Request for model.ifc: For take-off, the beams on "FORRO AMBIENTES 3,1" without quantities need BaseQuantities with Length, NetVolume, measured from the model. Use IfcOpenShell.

First a look at what the model holds.

```python
import ifcopenshell
import ifcopenshell.util.element
import ifcopenshell.util.unit

model = ifcopenshell.open("model.ifc")
print(model.schema)
for unit_type in ("LENGTHUNIT", "AREAUNIT", "VOLUMEUNIT"):
    print(unit_type, ifcopenshell.util.unit.calculate_unit_scale(model, unit_type))
storey = next(s for s in model.by_type("IfcBuildingStorey") if s.Name == "FORRO AMBIENTES 3,1")
beams = [e for e in ifcopenshell.util.element.get_decomposition(storey) if e.is_a("IfcBeam")]
for e in sorted(beams, key=lambda e: e.id()):
    print(e.id(), e.is_a(), e.Name, list(ifcopenshell.util.element.get_psets(e, qtos_only=True)), sep=" | ")
```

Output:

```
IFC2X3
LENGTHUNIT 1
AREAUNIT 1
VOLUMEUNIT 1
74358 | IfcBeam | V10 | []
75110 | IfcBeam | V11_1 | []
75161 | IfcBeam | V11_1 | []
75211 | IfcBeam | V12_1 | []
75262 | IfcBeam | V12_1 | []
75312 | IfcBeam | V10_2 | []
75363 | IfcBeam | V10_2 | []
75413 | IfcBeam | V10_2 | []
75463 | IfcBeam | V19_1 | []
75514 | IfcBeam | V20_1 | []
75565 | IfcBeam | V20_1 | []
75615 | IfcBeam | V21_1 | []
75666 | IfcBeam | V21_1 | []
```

```python
import ifcopenshell
import ifcopenshell.api.pset
import ifcopenshell.geom
import ifcopenshell.util.element
import ifcopenshell.util.shape
import ifcopenshell.util.unit

model = ifcopenshell.open("model.ifc")
unit_scale = ifcopenshell.util.unit.calculate_unit_scale(model)
volume_scale = ifcopenshell.util.unit.calculate_unit_scale(model, "VOLUMEUNIT")
settings = ifcopenshell.geom.settings()

storey = next(s for s in model.by_type("IfcBuildingStorey") if s.Name == "FORRO AMBIENTES 3,1")
beams = [e for e in ifcopenshell.util.element.get_decomposition(storey) if e.is_a("IfcBeam")]

for e in sorted(beams, key=lambda e: e.id()):
    if ifcopenshell.util.element.get_psets(e, qtos_only=True, should_inherit=False):
        continue
    # Geometry comes back in metres, in the element's own axes.
    shape = ifcopenshell.geom.create_shape(settings, e)
    values = {
        "Length": ifcopenshell.util.shape.get_max_xyz(shape.geometry) / unit_scale,
        "NetVolume": ifcopenshell.util.shape.get_volume(shape.geometry) / volume_scale,
    }
    qto = ifcopenshell.api.pset.add_qto(model, product=e, name="BaseQuantities")
    ifcopenshell.api.pset.edit_qto(model, qto=qto, properties=values)
    print(e.id(), {k: round(v, 3) for k, v in values.items()})

model.write("model_updated.ifc")
```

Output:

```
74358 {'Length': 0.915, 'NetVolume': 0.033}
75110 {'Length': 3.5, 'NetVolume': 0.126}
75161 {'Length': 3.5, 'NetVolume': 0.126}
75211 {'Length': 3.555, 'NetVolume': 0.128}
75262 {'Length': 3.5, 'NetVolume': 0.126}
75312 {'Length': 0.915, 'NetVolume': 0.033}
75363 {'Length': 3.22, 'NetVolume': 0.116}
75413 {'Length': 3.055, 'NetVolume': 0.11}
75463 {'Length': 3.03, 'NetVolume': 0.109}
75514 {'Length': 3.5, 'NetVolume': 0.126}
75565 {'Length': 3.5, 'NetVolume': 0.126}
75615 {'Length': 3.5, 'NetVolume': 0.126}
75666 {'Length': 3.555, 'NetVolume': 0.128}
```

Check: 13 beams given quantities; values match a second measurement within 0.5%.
